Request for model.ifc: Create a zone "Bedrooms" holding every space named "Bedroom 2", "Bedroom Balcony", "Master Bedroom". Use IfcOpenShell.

First a look at what the model holds.

```python
import ifcopenshell

model = ifcopenshell.open("model.ifc")
print(model.schema)
seen = {}
for space in model.by_type("IfcSpace"):
    seen[space.LongName] = seen.get(space.LongName, 0) + 1
for name, count in sorted(seen.items(), key=str):
    print(count, "x", name)
print("zones:", [z.Name for z in model.by_type("IfcZone")][:20])
```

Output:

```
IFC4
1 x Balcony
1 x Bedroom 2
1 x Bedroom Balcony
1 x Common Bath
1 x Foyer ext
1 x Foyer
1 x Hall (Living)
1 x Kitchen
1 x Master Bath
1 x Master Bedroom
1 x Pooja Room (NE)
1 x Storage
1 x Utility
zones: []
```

```python
import ifcopenshell
import ifcopenshell.api.group
import ifcopenshell.api.root

model = ifcopenshell.open("model.ifc")

names = {"Bedroom 2", "Bedroom Balcony", "Master Bedroom"}
spaces = [s for s in model.by_type("IfcSpace") if s.LongName in names]

zone = ifcopenshell.api.root.create_entity(model, ifc_class="IfcZone", name="Bedrooms")
ifcopenshell.api.group.assign_group(model, products=spaces, group=zone)
print(len(spaces), "spaces in", zone.Name)

model.write("model-out.ifc")
```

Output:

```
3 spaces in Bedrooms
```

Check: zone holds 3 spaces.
